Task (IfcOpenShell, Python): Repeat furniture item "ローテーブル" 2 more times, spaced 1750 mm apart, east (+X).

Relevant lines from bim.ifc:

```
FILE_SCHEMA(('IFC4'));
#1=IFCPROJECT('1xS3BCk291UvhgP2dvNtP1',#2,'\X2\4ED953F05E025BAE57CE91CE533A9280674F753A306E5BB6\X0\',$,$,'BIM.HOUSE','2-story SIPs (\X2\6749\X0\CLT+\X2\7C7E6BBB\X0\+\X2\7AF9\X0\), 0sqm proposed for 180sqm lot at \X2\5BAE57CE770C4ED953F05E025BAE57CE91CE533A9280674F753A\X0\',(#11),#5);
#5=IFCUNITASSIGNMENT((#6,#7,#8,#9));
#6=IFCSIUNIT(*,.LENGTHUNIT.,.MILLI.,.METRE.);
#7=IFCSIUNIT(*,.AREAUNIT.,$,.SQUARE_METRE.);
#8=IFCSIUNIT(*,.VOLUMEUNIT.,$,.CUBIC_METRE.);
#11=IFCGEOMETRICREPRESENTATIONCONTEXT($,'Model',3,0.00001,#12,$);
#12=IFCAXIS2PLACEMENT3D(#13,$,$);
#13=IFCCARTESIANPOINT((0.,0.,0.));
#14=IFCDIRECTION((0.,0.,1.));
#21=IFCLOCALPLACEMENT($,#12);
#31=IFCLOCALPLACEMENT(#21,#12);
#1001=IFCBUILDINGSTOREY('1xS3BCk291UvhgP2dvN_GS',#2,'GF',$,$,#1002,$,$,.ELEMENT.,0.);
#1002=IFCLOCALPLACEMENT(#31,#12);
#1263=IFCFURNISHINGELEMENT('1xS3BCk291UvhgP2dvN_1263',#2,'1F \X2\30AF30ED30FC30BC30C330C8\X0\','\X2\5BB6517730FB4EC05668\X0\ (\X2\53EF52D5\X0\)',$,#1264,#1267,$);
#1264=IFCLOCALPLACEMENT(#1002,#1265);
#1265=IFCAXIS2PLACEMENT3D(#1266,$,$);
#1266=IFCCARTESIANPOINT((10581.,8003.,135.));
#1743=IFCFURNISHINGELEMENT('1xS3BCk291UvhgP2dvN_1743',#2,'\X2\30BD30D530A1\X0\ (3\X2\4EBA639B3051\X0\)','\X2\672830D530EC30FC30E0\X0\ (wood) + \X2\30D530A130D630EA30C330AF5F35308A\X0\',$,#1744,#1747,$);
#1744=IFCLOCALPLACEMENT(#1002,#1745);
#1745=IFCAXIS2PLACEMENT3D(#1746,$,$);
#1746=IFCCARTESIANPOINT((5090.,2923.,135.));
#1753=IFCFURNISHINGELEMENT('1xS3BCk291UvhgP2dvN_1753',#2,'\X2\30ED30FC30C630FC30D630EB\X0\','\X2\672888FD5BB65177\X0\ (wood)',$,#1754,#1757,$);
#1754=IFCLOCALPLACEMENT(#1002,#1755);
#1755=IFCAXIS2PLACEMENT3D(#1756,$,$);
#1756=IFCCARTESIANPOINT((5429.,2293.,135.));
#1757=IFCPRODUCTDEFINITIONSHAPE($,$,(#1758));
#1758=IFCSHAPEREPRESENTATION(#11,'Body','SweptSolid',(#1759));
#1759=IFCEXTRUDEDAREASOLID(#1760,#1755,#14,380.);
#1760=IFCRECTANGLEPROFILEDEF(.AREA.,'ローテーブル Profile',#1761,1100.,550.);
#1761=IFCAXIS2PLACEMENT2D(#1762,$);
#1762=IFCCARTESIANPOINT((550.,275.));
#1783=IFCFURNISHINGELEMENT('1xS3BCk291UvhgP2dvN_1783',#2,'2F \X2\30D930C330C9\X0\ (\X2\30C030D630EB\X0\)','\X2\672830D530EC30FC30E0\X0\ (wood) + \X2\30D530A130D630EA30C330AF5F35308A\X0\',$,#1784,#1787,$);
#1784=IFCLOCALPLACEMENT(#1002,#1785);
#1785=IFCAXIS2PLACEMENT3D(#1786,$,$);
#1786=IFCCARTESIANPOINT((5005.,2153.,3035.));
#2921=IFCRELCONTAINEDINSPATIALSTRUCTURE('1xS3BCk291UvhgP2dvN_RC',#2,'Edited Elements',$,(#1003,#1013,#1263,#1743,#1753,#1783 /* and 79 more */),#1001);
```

```python
import numpy as np
import ifcopenshell
import ifcopenshell.api.geometry
import ifcopenshell.api.root
import ifcopenshell.util.element
import ifcopenshell.util.placement
import ifcopenshell.util.unit

model = ifcopenshell.open("bim.ifc")
unit_scale = ifcopenshell.util.unit.calculate_unit_scale(model)


def reuse_history(source, copy):
    """copy_class also copies each property set's owner history, people and application; keep the originals."""
    for rel in copy.IsDefinedBy:
        if rel.is_a("IfcRelDefinesByProperties") and (history := rel.RelatingPropertyDefinition.OwnerHistory):
            rel.RelatingPropertyDefinition.OwnerHistory = source.OwnerHistory
            ifcopenshell.util.element.remove_deep2(model, history)


source = model.by_guid("1xS3BCk291UvhgP2dvN_1753")
base = ifcopenshell.util.placement.get_local_placement(source.ObjectPlacement)
step = np.array([1.0, 0.0, 0.0]) * 1.75 / unit_scale

for i in range(1, 3):
    copy = ifcopenshell.api.root.copy_class(model, product=source)
    copy.Representation = ifcopenshell.util.element.copy_deep(
        model, source.Representation, exclude=["IfcGeometricRepresentationContext", "IfcRepresentationMap"]
    )
    reuse_history(source, copy)
    matrix = base.copy()
    matrix[:3, 3] += i * step
    print("added at", matrix[:3, 3].round(3) + 0.0)
    ifcopenshell.api.geometry.edit_object_placement(model, product=copy, matrix=matrix, is_si=False)

model.write("bim_edited.ifc")
```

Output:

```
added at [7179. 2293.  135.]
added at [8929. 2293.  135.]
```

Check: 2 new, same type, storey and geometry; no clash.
